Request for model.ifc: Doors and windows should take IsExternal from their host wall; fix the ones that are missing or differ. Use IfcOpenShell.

First a look at what the model holds.

```python
import ifcopenshell
import ifcopenshell.util.element

model = ifcopenshell.open("model.ifc")
print(model.schema)
seen = {}
for e in model.by_type("IfcDoor") + model.by_type("IfcWindow"):
    if not e.FillsVoids:
        continue
    host = e.FillsVoids[0].RelatingOpeningElement.VoidsElements[0].RelatingBuildingElement
    own = ifcopenshell.util.element.get_pset(e, f"Pset_{e.is_a()[3:].removesuffix('StandardCase')}Common", "IsExternal")
    wall = ifcopenshell.util.element.get_pset(host, "Pset_WallCommon", "IsExternal")
    seen[e.is_a(), own, wall] = seen.get((e.is_a(), own, wall), 0) + 1
for (cls, own, wall), count in sorted(seen.items(), key=str):
    print(count, cls, "IsExternal:", own, "| host wall:", wall)
```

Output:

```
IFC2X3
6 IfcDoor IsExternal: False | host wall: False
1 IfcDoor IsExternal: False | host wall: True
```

```python
import ifcopenshell
import ifcopenshell.api.pset
import ifcopenshell.util.element

model = ifcopenshell.open("model.ifc")

count = 0
for ifc_class, pset_name in (("IfcDoor", "Pset_DoorCommon"), ("IfcWindow", "Pset_WindowCommon")):
    for e in model.by_type(ifc_class):
        if not e.FillsVoids:
            continue
        host = e.FillsVoids[0].RelatingOpeningElement.VoidsElements[0].RelatingBuildingElement
        external = ifcopenshell.util.element.get_pset(host, "Pset_WallCommon", "IsExternal")
        if external is None or ifcopenshell.util.element.get_pset(e, pset_name, "IsExternal") == external:
            continue
        pset = ifcopenshell.api.pset.add_pset(model, product=e, name=pset_name)
        ifcopenshell.api.pset.edit_pset(model, pset=pset, properties={"IsExternal": external})
        count += 1

print(count, "updated")

model.write("model-out.ifc")
```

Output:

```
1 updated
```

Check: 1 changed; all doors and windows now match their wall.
